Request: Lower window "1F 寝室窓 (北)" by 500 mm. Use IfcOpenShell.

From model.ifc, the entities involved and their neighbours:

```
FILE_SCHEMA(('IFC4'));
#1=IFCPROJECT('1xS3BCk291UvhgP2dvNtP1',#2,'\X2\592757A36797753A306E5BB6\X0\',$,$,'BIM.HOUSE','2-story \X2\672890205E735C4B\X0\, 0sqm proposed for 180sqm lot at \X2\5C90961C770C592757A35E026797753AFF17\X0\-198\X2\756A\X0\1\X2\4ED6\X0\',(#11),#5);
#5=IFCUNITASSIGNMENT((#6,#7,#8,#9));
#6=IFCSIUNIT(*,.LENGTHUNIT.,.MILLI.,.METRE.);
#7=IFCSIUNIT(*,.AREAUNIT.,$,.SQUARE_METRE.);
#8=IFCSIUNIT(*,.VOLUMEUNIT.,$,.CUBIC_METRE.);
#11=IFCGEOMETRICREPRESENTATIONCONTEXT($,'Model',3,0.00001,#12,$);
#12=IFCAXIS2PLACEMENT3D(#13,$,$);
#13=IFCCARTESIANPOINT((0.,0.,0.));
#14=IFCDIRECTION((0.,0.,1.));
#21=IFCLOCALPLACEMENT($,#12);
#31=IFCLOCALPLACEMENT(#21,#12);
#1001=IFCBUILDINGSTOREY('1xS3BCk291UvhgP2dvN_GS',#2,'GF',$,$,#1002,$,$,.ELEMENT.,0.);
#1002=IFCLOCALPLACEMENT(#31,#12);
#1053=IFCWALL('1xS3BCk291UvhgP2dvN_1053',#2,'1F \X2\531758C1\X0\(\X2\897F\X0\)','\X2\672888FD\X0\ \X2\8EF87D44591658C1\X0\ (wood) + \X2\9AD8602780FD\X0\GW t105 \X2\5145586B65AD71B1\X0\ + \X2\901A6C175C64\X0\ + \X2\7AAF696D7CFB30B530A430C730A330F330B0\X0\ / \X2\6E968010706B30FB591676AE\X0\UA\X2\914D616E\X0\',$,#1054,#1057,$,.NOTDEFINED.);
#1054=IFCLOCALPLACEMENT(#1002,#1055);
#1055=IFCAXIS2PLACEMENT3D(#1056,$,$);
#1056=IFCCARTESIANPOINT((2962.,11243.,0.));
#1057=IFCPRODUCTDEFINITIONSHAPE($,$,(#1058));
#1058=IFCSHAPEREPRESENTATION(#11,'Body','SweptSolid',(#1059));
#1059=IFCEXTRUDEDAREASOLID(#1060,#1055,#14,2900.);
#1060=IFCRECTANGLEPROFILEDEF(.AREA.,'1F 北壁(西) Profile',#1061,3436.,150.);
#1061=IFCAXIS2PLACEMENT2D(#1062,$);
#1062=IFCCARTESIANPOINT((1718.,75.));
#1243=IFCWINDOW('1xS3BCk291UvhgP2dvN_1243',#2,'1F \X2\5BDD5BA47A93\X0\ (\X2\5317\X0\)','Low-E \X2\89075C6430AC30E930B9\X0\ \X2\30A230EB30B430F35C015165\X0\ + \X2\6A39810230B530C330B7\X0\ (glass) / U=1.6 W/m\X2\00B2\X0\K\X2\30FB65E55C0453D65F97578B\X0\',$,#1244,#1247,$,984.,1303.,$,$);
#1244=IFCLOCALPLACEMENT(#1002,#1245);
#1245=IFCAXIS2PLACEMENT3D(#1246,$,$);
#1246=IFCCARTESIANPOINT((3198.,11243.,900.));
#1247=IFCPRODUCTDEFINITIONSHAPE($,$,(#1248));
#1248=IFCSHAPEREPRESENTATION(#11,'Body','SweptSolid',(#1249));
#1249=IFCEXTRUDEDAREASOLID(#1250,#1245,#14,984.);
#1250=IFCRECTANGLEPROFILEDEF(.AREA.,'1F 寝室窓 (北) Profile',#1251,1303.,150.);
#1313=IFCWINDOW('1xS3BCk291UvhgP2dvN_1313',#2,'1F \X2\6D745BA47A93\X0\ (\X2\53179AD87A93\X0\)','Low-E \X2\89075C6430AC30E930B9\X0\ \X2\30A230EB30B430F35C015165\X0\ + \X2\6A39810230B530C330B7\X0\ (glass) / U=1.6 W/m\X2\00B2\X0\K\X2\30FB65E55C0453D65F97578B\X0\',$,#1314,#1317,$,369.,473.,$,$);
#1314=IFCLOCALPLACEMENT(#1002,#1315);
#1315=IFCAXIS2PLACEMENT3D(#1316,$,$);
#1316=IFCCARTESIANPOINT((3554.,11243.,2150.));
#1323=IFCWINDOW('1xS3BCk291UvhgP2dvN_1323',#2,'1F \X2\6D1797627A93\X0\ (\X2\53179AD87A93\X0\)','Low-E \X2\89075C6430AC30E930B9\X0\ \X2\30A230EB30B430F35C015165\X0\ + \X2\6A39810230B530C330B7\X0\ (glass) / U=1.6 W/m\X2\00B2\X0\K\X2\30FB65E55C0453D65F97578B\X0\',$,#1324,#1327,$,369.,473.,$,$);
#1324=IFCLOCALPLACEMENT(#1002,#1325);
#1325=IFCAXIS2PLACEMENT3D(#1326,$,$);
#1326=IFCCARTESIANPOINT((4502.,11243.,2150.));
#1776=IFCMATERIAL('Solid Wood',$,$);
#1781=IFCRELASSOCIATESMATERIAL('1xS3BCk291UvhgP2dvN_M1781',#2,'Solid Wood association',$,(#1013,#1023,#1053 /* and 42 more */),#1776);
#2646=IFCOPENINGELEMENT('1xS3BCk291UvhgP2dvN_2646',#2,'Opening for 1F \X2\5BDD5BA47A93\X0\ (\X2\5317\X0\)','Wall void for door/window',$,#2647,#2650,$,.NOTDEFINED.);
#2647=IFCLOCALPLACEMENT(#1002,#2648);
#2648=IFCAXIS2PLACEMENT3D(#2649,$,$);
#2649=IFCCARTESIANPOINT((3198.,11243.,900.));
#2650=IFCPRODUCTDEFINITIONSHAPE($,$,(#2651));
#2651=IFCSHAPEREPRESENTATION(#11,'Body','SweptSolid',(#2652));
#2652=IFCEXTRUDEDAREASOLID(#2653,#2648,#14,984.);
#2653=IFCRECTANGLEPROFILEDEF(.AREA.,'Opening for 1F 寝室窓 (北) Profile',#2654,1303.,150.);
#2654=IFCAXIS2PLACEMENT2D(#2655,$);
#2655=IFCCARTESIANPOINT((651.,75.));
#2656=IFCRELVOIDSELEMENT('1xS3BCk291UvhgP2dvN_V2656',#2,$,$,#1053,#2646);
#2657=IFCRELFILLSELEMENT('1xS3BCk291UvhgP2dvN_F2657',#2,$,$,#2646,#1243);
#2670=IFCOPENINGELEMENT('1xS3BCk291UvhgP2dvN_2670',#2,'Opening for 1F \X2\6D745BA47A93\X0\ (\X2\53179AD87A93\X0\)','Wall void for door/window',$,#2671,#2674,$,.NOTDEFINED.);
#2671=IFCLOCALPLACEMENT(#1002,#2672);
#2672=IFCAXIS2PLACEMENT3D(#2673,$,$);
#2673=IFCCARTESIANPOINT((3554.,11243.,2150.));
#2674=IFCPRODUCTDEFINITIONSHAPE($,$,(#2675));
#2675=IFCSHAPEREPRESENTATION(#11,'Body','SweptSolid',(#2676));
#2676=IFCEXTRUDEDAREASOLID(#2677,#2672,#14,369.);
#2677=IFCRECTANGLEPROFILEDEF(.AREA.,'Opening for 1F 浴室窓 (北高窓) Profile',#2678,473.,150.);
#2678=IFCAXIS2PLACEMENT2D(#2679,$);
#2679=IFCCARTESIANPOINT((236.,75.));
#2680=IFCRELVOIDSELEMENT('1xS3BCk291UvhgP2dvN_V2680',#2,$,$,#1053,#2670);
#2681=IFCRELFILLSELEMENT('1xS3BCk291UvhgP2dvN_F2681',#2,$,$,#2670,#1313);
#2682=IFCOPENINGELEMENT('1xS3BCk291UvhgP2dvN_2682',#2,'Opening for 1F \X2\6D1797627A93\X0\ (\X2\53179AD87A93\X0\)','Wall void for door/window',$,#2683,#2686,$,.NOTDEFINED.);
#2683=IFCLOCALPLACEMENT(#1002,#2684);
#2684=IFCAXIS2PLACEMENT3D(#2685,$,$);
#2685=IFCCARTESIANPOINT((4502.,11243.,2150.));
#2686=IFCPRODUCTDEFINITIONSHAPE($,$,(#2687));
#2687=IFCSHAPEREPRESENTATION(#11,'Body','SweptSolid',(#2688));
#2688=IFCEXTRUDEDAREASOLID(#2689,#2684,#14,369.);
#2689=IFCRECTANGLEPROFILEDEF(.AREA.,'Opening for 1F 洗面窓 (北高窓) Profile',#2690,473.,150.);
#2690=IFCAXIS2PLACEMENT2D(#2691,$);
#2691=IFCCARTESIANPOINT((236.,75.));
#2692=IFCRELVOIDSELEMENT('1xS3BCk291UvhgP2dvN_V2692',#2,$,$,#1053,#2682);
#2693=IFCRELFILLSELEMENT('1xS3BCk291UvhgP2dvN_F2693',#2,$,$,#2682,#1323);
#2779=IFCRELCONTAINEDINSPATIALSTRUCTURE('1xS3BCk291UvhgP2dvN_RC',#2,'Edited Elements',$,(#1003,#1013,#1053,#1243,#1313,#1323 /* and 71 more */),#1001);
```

```python
import numpy as np
import ifcopenshell
import ifcopenshell.api.geometry
import ifcopenshell.util.placement
import ifcopenshell.util.unit

model = ifcopenshell.open("model.ifc")
unit_scale = ifcopenshell.util.unit.calculate_unit_scale(model)

window = model.by_guid("1xS3BCk291UvhgP2dvN_1243")
opening = window.FillsVoids[0].RelatingOpeningElement
dz = -0.5 / unit_scale

shift = np.array([0.0, 0.0, dz])
# The window is not placed relative to its opening, so move both.
for product in (opening, window):
    matrix = ifcopenshell.util.placement.get_local_placement(product.ObjectPlacement)
    matrix[:3, 3] += shift
    ifcopenshell.api.geometry.edit_object_placement(model, product=product, matrix=matrix, is_si=False)

print(f"moved by {dz * unit_scale:+.3f} m")

model.write("model_edited.ifc")
```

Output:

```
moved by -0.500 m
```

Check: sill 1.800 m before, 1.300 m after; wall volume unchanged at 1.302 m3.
